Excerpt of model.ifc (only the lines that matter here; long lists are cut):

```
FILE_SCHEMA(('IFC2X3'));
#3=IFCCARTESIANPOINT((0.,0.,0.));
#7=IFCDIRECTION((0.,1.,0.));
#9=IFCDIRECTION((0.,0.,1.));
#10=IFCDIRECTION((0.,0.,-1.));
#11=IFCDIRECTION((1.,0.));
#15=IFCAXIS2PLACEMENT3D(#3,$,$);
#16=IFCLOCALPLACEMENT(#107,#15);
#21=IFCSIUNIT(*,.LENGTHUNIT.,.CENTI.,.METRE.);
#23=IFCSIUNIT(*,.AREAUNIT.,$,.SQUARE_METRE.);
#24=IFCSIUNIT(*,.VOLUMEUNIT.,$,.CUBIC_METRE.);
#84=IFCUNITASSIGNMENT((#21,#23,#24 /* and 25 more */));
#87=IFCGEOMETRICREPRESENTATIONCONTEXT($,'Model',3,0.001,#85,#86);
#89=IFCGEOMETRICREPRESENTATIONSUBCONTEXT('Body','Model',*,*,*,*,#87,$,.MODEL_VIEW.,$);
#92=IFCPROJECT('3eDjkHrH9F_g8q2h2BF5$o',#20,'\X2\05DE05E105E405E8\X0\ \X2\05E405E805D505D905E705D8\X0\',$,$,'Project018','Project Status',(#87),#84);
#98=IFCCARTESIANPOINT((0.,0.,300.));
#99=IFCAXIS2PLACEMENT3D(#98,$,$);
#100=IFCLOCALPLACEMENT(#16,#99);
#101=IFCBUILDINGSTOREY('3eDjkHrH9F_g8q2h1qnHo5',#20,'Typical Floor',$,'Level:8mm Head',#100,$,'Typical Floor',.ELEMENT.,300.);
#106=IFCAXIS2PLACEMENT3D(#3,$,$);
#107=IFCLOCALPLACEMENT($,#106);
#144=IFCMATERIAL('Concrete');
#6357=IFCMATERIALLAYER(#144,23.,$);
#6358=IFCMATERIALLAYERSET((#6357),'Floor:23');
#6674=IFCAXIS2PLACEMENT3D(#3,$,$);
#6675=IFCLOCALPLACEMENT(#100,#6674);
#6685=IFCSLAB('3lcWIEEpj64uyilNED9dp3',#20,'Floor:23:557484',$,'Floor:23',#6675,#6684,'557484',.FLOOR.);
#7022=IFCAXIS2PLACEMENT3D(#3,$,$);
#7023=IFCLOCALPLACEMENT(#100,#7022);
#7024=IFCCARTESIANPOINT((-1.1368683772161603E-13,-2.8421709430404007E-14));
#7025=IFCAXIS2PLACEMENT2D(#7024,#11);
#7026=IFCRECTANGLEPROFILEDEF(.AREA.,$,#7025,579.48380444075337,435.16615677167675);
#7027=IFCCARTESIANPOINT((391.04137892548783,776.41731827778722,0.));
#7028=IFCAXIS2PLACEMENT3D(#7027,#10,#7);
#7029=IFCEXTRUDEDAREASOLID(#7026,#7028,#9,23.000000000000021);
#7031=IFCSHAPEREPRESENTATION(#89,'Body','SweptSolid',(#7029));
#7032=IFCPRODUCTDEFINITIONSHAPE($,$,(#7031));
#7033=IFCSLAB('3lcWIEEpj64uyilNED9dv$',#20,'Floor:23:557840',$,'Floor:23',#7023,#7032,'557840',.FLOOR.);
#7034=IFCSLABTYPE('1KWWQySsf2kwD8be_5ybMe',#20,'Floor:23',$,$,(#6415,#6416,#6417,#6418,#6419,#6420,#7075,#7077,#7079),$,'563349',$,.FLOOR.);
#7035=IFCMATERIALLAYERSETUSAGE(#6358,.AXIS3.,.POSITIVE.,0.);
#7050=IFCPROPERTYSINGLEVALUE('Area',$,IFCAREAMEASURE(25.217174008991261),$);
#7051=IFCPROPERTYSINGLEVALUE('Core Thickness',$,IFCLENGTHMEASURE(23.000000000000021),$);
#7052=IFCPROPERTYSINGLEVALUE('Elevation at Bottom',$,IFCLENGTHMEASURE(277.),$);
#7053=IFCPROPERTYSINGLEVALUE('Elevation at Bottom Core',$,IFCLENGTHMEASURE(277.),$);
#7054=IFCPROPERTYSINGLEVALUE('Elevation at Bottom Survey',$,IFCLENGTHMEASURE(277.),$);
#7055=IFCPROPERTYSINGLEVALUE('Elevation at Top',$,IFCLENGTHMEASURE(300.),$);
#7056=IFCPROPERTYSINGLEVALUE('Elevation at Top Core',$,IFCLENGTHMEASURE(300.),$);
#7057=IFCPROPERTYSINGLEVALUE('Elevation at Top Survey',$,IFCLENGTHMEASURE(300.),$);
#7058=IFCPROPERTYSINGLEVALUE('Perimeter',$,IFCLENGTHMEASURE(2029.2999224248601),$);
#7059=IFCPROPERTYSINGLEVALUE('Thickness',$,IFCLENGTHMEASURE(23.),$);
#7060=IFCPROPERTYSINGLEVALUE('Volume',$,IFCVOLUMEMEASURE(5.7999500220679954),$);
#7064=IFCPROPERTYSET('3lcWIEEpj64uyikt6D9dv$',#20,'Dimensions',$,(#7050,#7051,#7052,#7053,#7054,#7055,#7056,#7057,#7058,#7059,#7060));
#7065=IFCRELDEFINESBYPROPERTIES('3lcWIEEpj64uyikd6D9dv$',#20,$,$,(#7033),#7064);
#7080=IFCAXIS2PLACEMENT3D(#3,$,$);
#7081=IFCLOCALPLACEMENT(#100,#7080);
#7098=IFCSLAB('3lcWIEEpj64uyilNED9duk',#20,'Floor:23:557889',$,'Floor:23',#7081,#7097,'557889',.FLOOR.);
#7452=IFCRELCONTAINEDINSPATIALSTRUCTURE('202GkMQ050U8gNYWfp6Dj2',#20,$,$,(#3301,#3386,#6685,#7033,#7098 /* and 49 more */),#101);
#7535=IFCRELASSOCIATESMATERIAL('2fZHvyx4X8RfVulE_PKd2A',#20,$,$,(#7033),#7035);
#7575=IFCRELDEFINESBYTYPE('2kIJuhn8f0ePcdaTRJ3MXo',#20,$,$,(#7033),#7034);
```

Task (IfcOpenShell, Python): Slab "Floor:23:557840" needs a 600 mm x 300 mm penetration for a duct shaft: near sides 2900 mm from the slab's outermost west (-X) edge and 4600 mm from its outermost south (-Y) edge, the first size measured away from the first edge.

```python
import numpy as np
import ifcopenshell
import ifcopenshell.api.feature
import ifcopenshell.api.geometry
import ifcopenshell.api.pset
import ifcopenshell.api.root
import ifcopenshell.geom
import ifcopenshell.util.element
import ifcopenshell.util.placement
import ifcopenshell.util.representation
import ifcopenshell.util.shape
import ifcopenshell.util.unit

model = ifcopenshell.open("model.ifc")
unit_scale = ifcopenshell.util.unit.calculate_unit_scale(model)
area_scale = ifcopenshell.util.unit.calculate_unit_scale(model, "AREAUNIT")
volume_scale = ifcopenshell.util.unit.calculate_unit_scale(model, "VOLUMEUNIT")
settings = ifcopenshell.geom.settings()


def volume(element):
    """Net volume in cubic metres, openings subtracted."""
    shape = ifcopenshell.geom.create_shape(settings, element)
    return ifcopenshell.util.shape.get_volume(shape.geometry)


slab = model.by_guid("3lcWIEEpj64uyilNED9dv$")
before = volume(slab)

# Extent in the slab's own axes, in metres. The edges named are its -X and -Y sides.
slab_shape = ifcopenshell.geom.create_shape(settings, slab)
vertices = ifcopenshell.util.shape.get_vertices(slab_shape.geometry)
x_min, y_min, bottom = vertices.min(axis=0)
top = vertices[:, 2].max()

opening = ifcopenshell.api.root.create_entity(model, ifc_class="IfcOpeningElement", name="Duct shaft opening")
context = ifcopenshell.util.representation.get_context(model, "Model", "Body", "MODEL_VIEW")
width, depth = 0.6, 0.3
outline = [(0.0, 0.0), (width, 0.0), (width, depth), (0.0, depth), (0.0, 0.0)]
# Overshoot both faces by 50 mm so the cut is clean.
shape = ifcopenshell.api.geometry.add_slab_representation(
    model, context=context, depth=top - bottom + 0.1, polyline=outline
)
ifcopenshell.api.geometry.assign_representation(model, product=opening, representation=shape)

matrix = ifcopenshell.util.placement.get_local_placement(slab.ObjectPlacement)
matrix[:, 3] = matrix @ np.append(np.array([x_min + 2.9, y_min + 4.6, bottom - 0.05]) / unit_scale, 1.0)
ifcopenshell.api.geometry.edit_object_placement(model, product=opening, matrix=matrix, is_si=False)
ifcopenshell.api.feature.add_feature(model, feature=opening, element=slab)

after = volume(slab)

# Update the slab's stored quantities.
pset = model.by_id(ifcopenshell.util.element.get_pset(slab, "Dimensions", should_inherit=False)["id"])
ifcopenshell.api.pset.edit_pset(model, pset=pset, properties={
    "Area": model.create_entity("IfcAreaMeasure", after / (top - bottom) / area_scale),
    "Volume": model.create_entity("IfcVolumeMeasure", after / volume_scale),
})

print(f"slab volume {before:.3f} -> {after:.3f} m3")

model.write("model-out.ifc")
```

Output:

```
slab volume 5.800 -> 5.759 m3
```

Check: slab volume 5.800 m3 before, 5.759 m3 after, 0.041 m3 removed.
